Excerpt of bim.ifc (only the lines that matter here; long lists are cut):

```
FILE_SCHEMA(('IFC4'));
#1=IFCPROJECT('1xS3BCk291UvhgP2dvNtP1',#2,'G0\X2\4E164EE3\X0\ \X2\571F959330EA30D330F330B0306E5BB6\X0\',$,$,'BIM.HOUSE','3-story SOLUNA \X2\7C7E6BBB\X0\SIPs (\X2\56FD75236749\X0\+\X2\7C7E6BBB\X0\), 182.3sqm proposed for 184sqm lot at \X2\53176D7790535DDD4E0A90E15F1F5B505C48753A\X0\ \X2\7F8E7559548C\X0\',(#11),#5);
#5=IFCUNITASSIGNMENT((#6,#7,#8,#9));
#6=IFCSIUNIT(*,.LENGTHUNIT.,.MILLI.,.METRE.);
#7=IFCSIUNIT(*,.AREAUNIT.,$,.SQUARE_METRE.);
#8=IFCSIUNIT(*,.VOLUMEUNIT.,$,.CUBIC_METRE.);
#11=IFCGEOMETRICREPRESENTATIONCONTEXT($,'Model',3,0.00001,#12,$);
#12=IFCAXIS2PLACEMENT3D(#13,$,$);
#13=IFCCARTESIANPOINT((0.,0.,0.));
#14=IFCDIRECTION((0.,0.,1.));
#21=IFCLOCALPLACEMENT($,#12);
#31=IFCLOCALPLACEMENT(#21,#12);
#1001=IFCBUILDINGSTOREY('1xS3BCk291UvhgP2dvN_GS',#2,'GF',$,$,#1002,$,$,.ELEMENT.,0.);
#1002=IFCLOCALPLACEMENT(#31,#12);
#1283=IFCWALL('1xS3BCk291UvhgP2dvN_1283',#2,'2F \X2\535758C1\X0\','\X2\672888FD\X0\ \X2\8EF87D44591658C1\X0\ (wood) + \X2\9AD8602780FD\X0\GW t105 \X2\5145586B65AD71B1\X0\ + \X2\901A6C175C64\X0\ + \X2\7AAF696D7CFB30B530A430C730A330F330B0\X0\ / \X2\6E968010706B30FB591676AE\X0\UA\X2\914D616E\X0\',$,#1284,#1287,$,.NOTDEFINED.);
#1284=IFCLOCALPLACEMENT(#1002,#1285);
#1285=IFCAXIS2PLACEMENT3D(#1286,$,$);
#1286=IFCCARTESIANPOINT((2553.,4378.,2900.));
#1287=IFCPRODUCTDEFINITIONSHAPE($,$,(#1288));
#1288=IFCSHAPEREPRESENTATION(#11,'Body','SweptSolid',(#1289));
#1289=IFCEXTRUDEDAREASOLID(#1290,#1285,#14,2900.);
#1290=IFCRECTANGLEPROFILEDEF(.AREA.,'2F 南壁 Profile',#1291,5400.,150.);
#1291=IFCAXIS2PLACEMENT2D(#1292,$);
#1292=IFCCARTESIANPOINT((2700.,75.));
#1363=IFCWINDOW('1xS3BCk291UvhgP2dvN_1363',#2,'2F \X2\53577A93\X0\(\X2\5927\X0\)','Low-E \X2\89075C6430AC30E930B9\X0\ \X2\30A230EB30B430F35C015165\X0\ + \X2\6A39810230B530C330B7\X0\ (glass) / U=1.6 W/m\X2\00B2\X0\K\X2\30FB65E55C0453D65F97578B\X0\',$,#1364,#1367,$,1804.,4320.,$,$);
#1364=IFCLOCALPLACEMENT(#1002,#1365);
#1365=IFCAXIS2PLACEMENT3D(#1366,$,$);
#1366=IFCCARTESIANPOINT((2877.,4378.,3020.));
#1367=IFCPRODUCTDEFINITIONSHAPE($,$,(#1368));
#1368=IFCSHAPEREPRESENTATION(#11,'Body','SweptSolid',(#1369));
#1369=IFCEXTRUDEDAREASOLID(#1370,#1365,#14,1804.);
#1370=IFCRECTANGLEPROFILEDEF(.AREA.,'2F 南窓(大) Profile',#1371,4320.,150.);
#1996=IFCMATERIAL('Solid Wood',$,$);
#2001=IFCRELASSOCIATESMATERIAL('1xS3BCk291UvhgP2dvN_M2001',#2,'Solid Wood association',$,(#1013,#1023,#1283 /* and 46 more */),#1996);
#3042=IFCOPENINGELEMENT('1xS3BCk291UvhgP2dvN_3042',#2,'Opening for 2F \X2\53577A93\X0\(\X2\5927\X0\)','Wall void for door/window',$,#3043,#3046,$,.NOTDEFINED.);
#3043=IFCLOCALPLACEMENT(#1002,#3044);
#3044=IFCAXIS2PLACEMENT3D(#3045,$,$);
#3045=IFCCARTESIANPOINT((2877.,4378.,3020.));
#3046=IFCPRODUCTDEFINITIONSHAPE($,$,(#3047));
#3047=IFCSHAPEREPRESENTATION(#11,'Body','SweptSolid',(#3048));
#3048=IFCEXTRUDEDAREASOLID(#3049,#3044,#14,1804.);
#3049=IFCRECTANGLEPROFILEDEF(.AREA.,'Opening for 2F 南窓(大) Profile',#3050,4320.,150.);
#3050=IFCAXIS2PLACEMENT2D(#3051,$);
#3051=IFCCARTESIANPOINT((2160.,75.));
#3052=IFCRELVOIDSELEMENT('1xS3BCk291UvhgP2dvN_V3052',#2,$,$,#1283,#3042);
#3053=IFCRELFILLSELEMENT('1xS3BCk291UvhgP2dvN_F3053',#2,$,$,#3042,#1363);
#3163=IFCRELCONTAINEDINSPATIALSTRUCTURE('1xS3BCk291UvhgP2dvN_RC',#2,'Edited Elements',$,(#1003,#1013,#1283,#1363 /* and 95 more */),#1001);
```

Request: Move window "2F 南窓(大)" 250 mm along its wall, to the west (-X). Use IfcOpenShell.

```python
import ifcopenshell
import ifcopenshell.api.geometry
import ifcopenshell.util.placement
import ifcopenshell.util.unit

model = ifcopenshell.open("bim.ifc")
unit_scale = ifcopenshell.util.unit.calculate_unit_scale(model)

window = model.by_guid("1xS3BCk291UvhgP2dvN_1363")
opening = window.FillsVoids[0].RelatingOpeningElement
wall = opening.VoidsElements[0].RelatingBuildingElement

wall_matrix = ifcopenshell.util.placement.get_local_placement(wall.ObjectPlacement)
shift = wall_matrix[:3, 0] * -0.25 / unit_scale
before = ifcopenshell.util.placement.get_local_placement(window.ObjectPlacement)[:3, 3].copy()

# The window is not placed relative to its opening, so move both.
for product in (opening, window):
    matrix = ifcopenshell.util.placement.get_local_placement(product.ObjectPlacement)
    matrix[:3, 3] += shift
    ifcopenshell.api.geometry.edit_object_placement(model, product=product, matrix=matrix, is_si=False)

after = ifcopenshell.util.placement.get_local_placement(window.ObjectPlacement)[:3, 3]
print("window moved by", (after - before).round(3) + 0.0)

model.write("bim-out.ifc")
```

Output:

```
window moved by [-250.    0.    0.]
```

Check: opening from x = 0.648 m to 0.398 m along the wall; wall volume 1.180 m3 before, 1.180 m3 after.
